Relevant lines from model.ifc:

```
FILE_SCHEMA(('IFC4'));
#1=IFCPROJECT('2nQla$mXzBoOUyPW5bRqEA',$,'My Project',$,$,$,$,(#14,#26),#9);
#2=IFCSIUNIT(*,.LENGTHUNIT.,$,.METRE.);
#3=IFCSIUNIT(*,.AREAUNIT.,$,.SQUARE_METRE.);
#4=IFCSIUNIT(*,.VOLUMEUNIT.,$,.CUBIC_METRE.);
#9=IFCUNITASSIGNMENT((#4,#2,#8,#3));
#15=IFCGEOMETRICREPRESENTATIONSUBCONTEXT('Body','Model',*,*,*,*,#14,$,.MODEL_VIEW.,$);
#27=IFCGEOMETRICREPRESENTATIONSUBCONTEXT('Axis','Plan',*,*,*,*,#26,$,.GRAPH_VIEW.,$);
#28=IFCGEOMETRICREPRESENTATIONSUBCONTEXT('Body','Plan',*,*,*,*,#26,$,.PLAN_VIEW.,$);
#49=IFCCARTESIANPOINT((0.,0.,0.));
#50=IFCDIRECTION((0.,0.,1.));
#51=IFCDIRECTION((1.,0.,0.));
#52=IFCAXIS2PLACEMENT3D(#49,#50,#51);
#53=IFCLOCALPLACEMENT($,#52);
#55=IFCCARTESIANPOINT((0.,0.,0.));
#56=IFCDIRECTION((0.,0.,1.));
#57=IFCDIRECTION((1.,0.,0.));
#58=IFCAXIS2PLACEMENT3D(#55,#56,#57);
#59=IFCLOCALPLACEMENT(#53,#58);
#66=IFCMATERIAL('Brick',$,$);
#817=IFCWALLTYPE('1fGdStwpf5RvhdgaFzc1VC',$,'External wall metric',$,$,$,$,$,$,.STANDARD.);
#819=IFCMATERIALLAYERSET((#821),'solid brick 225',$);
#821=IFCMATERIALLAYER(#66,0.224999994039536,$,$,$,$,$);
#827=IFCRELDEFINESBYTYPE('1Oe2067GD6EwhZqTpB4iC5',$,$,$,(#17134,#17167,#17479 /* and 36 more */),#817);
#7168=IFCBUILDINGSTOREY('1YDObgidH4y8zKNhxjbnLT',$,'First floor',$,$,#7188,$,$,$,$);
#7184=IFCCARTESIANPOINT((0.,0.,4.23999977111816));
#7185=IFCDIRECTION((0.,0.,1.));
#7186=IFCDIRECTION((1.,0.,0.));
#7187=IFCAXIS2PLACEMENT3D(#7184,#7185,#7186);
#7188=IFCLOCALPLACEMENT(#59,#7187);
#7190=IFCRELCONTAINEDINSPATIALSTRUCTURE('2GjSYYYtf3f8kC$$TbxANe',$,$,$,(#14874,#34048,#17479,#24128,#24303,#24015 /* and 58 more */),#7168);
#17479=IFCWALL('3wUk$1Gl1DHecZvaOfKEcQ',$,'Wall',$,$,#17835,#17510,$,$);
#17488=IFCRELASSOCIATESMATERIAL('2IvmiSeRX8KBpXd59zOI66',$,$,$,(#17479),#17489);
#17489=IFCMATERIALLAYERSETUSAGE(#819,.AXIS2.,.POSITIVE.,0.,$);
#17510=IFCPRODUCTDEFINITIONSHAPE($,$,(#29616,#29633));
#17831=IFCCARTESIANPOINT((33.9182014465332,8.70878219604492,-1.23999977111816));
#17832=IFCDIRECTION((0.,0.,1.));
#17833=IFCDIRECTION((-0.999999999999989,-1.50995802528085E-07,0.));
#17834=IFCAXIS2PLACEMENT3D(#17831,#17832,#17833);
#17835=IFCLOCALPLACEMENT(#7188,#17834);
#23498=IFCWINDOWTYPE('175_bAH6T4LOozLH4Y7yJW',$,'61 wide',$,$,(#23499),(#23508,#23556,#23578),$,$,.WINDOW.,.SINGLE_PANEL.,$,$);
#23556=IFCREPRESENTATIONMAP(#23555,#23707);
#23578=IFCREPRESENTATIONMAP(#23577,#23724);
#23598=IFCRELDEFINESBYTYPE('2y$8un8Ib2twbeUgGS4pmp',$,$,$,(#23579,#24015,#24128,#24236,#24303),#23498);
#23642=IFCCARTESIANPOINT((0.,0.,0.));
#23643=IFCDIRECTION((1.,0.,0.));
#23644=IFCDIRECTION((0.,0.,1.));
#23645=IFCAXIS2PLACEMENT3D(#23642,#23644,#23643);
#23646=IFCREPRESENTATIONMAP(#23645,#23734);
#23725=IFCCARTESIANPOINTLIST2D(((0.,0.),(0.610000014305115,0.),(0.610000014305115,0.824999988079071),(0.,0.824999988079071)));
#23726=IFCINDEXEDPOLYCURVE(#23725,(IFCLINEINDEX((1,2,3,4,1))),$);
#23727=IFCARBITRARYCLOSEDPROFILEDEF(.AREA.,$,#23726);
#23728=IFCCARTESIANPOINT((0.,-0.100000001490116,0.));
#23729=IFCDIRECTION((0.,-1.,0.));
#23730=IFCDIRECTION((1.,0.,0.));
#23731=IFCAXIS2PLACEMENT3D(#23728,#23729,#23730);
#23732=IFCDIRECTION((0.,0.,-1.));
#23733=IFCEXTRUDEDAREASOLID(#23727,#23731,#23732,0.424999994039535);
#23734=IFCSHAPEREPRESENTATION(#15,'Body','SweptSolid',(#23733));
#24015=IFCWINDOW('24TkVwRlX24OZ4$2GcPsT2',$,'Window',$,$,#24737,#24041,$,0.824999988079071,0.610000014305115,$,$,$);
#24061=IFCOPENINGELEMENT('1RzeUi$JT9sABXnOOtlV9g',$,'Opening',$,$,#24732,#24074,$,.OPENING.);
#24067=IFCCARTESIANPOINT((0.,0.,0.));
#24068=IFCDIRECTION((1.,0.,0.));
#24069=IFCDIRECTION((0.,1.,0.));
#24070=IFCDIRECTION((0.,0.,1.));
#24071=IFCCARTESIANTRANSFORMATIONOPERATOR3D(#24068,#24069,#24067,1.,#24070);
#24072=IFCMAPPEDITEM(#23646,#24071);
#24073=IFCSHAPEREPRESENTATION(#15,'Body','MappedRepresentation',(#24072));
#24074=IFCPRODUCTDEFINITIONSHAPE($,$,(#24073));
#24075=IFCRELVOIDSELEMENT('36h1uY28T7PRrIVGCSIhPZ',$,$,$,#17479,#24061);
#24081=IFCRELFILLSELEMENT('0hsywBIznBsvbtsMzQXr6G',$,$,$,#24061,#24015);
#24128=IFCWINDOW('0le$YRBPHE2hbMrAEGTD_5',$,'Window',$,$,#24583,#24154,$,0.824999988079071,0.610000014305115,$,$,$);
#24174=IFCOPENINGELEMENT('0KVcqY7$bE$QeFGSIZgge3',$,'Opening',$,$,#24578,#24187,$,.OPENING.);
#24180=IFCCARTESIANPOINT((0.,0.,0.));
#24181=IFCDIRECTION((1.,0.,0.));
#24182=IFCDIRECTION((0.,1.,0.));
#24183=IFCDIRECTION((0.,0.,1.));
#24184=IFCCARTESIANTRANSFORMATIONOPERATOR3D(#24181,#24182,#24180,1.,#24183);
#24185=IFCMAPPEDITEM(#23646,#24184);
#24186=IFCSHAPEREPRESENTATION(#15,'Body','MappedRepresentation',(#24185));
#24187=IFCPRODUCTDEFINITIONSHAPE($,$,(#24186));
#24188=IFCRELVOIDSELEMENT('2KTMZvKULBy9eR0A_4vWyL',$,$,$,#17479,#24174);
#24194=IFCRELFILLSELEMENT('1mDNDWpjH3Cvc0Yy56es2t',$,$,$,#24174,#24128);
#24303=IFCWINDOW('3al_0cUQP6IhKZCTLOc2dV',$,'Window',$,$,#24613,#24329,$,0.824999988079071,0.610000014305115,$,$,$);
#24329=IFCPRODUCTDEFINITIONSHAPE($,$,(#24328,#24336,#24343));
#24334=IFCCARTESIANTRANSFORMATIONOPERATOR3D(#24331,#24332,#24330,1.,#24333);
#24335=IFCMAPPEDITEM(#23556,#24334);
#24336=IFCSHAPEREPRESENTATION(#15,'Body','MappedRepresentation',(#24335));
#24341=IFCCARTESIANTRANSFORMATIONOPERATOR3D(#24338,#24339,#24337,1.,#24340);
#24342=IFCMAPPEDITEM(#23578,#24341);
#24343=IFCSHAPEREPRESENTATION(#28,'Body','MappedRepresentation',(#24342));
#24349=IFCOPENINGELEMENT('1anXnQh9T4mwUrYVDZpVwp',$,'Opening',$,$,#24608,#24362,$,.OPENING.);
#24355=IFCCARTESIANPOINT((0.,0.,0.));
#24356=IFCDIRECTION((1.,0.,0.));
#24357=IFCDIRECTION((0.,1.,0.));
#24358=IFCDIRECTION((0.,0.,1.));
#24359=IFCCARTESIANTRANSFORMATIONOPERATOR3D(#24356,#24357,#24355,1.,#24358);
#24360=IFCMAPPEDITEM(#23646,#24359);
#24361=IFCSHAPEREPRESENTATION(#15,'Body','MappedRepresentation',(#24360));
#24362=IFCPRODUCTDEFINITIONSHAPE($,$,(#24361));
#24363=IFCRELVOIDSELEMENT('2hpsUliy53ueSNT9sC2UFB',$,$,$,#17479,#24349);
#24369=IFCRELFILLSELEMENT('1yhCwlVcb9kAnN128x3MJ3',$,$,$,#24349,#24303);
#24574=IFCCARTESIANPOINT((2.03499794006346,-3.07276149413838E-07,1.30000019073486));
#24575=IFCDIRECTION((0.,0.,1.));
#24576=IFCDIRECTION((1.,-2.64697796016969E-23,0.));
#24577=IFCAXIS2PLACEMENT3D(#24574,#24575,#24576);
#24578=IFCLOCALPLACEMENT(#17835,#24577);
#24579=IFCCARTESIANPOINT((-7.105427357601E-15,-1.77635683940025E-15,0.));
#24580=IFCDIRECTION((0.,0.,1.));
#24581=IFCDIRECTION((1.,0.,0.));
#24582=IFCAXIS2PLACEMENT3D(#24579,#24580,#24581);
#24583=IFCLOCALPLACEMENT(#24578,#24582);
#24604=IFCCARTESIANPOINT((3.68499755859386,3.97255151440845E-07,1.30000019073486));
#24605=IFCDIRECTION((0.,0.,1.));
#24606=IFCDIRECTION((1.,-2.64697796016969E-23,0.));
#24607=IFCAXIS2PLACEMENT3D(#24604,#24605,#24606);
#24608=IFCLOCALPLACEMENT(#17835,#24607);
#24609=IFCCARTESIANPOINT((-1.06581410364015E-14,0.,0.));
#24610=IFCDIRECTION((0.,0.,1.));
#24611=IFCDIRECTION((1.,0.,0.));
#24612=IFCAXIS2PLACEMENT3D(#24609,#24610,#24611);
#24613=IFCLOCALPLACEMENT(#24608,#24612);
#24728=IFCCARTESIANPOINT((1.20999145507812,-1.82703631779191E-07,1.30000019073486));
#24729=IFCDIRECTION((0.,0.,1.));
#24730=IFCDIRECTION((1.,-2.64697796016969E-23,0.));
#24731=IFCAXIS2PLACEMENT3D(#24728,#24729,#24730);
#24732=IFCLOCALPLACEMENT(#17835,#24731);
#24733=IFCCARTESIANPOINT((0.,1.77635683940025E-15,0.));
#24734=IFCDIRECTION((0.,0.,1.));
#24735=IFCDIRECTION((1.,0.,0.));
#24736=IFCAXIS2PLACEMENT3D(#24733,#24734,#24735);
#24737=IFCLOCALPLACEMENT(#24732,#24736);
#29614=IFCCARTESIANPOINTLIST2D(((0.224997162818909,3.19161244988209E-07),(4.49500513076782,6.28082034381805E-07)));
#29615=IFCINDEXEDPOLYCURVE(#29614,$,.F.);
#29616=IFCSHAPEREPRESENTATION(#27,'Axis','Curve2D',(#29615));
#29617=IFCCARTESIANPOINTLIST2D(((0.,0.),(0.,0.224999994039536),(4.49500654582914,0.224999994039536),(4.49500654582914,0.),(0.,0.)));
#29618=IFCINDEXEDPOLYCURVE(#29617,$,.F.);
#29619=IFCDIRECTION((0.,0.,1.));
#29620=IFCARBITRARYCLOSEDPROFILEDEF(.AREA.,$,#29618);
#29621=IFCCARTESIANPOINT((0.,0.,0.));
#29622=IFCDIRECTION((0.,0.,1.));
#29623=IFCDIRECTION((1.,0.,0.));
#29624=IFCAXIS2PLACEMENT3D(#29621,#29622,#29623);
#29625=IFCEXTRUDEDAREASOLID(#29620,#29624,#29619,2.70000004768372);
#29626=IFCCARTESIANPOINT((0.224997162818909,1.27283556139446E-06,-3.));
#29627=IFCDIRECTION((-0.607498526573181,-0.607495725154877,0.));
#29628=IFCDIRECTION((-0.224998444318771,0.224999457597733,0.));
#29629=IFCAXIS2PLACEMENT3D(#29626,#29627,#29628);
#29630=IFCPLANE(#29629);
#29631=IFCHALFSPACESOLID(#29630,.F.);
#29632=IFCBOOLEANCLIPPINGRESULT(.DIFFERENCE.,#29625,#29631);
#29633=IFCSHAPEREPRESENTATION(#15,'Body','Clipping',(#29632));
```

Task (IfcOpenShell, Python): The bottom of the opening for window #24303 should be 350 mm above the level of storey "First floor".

```python
import numpy as np
import ifcopenshell
import ifcopenshell.api.geometry
import ifcopenshell.geom
import ifcopenshell.util.element
import ifcopenshell.util.placement
import ifcopenshell.util.shape
import ifcopenshell.util.unit

model = ifcopenshell.open("model.ifc")
unit_scale = ifcopenshell.util.unit.calculate_unit_scale(model)

window = model.by_guid("3al_0cUQP6IhKZCTLOc2dV")
opening = window.FillsVoids[0].RelatingOpeningElement
storey = ifcopenshell.util.element.get_container(window, ifc_class="IfcBuildingStorey")
level = ifcopenshell.util.placement.get_local_placement(storey.ObjectPlacement)[2, 3]

# The opening's origin need not be at the sill, so measure its lowest point.
shape = ifcopenshell.geom.create_shape(ifcopenshell.geom.settings(), opening)
bottom = ifcopenshell.util.shape.get_shape_bottom_elevation(shape, shape.geometry) / unit_scale
dz = level + 0.35 / unit_scale - bottom

shift = np.array([0.0, 0.0, dz])
# The window is placed relative to its opening, so it follows when the opening moves.
matrix = ifcopenshell.util.placement.get_local_placement(opening.ObjectPlacement)
matrix[:3, 3] += shift
ifcopenshell.api.geometry.edit_object_placement(
    model, product=opening, matrix=matrix, is_si=False, should_transform_children=True
)

print(f"moved by {dz * unit_scale:+.3f} m")

model.write("model-out.ifc")
```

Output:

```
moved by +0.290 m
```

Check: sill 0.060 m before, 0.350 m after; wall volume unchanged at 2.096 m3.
